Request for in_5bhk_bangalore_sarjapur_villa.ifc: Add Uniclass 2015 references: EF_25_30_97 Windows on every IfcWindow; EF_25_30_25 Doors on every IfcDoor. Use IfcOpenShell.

First a look at what the model holds.

```python
import ifcopenshell

model = ifcopenshell.open("in_5bhk_bangalore_sarjapur_villa.ifc")
print(model.schema)
print("classifications:", [c.Name for c in model.by_type("IfcClassification")])
for ifc_class in ("IfcDoor", "IfcRoof", "IfcStair", "IfcWall", "IfcWindow"):
    print(ifc_class, len(model.by_type(ifc_class)))
```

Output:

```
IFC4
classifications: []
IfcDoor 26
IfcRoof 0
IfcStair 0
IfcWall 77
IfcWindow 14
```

```python
import ifcopenshell
import ifcopenshell.api.classification

model = ifcopenshell.open("in_5bhk_bangalore_sarjapur_villa.ifc")

system = ifcopenshell.api.classification.add_classification(model, classification="Uniclass 2015")

codes = {
    "IfcWindow": ("EF_25_30_97", "Windows"),
    "IfcDoor": ("EF_25_30_25", "Doors"),
}
for ifc_class, (code, name) in codes.items():
    products = model.by_type(ifc_class)
    ifcopenshell.api.classification.add_reference(
        model, products=products, classification=system, identification=code, name=name
    )
    print(code, len(products))

model.write("in_5bhk_bangalore_sarjapur_villa_v2.ifc")
```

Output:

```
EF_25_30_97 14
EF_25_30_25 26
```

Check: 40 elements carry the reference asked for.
